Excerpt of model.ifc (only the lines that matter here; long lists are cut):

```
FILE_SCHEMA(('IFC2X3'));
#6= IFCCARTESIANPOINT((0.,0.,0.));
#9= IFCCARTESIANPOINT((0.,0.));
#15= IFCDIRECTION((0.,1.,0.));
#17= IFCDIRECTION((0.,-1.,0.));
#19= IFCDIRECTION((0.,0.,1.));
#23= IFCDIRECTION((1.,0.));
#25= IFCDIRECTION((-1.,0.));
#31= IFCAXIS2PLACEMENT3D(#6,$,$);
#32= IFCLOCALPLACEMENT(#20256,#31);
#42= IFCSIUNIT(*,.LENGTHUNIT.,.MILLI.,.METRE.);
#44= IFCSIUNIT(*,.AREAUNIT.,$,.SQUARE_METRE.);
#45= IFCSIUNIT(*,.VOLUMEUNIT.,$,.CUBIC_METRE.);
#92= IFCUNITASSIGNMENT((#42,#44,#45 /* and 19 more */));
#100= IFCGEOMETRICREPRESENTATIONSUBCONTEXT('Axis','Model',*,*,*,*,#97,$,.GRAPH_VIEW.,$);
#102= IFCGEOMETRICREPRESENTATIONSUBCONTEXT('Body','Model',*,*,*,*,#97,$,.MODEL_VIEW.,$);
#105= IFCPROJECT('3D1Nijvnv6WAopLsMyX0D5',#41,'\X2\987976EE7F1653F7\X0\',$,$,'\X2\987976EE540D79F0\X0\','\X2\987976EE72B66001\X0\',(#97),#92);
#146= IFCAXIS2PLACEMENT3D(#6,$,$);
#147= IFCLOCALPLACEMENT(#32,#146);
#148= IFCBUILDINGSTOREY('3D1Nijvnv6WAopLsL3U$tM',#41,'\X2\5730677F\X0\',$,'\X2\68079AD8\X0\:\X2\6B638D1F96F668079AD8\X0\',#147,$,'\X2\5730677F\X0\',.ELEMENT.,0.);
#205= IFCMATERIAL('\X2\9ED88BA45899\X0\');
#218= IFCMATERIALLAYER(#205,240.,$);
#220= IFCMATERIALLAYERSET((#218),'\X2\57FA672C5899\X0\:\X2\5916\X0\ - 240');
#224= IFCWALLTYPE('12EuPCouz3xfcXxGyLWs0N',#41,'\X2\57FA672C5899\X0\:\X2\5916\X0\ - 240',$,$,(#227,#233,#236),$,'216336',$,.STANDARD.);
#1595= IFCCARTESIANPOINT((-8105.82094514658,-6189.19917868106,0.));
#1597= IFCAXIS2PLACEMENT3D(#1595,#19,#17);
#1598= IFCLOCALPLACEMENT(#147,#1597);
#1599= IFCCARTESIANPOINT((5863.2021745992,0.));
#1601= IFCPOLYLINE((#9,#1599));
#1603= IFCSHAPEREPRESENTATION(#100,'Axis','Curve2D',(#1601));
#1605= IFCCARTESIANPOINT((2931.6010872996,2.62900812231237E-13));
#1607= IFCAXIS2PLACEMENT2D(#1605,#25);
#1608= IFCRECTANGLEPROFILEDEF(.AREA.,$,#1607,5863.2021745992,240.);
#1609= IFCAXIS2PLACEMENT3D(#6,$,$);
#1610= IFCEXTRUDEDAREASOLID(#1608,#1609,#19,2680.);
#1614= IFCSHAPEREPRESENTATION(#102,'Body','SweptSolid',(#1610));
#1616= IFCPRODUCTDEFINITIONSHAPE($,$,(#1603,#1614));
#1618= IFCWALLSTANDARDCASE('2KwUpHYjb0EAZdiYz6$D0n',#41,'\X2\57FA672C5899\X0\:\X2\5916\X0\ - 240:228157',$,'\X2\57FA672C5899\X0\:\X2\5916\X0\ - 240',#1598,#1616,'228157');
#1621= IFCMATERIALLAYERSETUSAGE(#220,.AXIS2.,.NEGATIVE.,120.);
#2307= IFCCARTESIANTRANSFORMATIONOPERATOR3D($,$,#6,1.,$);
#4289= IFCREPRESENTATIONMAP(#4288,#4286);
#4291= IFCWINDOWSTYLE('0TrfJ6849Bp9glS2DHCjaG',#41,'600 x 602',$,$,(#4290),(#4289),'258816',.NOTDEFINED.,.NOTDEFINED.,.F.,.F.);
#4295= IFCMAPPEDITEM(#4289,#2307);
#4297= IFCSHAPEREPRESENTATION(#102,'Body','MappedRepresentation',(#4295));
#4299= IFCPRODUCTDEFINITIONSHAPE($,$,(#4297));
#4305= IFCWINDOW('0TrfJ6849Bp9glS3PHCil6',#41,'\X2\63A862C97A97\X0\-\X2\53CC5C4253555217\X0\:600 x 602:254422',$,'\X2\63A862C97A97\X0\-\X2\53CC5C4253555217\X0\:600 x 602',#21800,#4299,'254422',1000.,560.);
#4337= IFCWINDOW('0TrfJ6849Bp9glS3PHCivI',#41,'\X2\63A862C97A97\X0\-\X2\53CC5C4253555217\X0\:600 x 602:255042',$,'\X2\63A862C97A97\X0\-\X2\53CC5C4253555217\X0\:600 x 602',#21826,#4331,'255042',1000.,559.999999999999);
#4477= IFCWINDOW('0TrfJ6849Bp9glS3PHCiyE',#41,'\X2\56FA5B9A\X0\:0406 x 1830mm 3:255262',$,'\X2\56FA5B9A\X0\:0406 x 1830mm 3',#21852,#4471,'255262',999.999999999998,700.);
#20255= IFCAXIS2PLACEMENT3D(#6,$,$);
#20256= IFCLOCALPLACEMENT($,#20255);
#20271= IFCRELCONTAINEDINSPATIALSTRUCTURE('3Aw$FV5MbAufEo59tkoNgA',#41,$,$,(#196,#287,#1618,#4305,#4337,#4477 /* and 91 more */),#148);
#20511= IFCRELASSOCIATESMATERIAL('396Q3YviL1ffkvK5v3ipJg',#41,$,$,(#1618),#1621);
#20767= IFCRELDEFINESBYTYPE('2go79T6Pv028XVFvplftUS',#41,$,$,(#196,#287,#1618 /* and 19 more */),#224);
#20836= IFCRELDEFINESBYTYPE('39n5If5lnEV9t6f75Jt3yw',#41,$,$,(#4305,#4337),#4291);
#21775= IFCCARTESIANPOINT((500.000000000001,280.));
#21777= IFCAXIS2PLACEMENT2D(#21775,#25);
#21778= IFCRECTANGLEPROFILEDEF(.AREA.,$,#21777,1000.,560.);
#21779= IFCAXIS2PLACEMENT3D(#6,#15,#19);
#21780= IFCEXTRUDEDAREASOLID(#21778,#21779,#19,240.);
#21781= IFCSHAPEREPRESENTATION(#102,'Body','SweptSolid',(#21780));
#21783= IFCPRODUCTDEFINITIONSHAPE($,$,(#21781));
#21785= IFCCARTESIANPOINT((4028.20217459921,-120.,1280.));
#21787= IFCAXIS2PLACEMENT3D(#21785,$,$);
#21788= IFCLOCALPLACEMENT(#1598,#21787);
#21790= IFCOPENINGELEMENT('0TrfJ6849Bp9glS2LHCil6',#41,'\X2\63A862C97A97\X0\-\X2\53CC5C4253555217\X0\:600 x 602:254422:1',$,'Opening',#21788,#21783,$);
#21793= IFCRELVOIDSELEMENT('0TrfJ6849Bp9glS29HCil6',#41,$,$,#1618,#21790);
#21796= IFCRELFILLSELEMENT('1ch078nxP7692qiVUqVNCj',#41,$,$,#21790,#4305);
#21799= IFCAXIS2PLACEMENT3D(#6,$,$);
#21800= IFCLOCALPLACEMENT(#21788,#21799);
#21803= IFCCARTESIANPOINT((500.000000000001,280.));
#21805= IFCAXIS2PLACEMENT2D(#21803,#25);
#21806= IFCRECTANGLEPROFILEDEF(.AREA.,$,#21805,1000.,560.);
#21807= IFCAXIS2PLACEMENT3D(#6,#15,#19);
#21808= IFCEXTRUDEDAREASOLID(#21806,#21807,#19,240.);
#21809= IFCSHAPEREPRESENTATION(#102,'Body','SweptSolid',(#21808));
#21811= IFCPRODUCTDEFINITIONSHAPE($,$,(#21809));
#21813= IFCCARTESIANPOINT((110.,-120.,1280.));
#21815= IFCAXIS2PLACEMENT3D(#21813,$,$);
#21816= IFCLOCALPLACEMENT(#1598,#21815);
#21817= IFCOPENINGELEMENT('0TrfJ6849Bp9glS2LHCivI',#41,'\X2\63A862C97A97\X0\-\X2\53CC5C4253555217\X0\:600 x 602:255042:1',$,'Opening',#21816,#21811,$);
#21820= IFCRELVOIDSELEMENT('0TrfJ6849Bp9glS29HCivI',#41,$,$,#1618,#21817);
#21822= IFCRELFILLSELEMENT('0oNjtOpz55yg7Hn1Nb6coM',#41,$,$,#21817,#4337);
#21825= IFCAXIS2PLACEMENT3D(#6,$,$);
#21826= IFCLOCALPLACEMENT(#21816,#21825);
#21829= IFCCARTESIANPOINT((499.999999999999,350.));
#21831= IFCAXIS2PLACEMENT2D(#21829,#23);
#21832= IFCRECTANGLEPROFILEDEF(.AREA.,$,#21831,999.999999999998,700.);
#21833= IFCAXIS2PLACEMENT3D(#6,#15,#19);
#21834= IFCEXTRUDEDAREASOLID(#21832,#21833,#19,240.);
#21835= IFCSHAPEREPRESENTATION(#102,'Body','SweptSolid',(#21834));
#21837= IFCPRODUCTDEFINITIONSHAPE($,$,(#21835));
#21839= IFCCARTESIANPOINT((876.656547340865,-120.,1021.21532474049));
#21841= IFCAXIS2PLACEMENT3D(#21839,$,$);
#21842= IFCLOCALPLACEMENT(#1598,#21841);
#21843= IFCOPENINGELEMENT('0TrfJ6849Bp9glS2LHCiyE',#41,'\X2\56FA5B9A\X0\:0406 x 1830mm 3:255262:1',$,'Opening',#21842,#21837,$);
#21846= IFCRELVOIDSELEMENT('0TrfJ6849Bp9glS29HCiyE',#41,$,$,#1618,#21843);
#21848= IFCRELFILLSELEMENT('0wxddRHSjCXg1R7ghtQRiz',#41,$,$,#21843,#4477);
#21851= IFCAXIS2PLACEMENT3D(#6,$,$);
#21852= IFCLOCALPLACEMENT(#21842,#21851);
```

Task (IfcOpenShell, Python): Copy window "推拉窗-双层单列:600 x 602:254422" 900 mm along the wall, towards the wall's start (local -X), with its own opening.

```python
import ifcopenshell
import ifcopenshell.api.feature
import ifcopenshell.api.geometry
import ifcopenshell.api.root
import ifcopenshell.geom
import ifcopenshell.util.element
import ifcopenshell.util.placement
import ifcopenshell.util.shape
import ifcopenshell.util.unit

model = ifcopenshell.open("model.ifc")
unit_scale = ifcopenshell.util.unit.calculate_unit_scale(model)
settings = ifcopenshell.geom.settings()


def volume(element):
    """Net volume in cubic metres, openings subtracted."""
    shape = ifcopenshell.geom.create_shape(settings, element)
    return ifcopenshell.util.shape.get_volume(shape.geometry)


def reuse_history(source, copy):
    """copy_class also copies each property set's owner history, people and application; keep the originals."""
    for rel in copy.IsDefinedBy:
        if rel.is_a("IfcRelDefinesByProperties") and (history := rel.RelatingPropertyDefinition.OwnerHistory):
            rel.RelatingPropertyDefinition.OwnerHistory = source.OwnerHistory
            ifcopenshell.util.element.remove_deep2(model, history)


window = model.by_guid("0TrfJ6849Bp9glS3PHCil6")
opening = window.FillsVoids[0].RelatingOpeningElement
wall = opening.VoidsElements[0].RelatingBuildingElement
before = volume(wall)
shift = ifcopenshell.util.placement.get_local_placement(wall.ObjectPlacement)[:3, 0] * -0.9 / unit_scale

# copy_class copies the void relationship, type, container and properties, but no geometry.
new_opening = ifcopenshell.api.root.copy_class(model, product=opening)
new_opening.Representation = ifcopenshell.util.element.copy_deep(
    model, opening.Representation, exclude=["IfcGeometricRepresentationContext", "IfcRepresentationMap"]
)
new_opening.Name = "推拉窗-双层单列:600 x 602"
new_window = ifcopenshell.api.root.copy_class(model, product=window)
new_window.Representation = ifcopenshell.util.element.copy_deep(
    model, window.Representation, exclude=["IfcGeometricRepresentationContext", "IfcRepresentationMap"]
)
new_window.Name = "推拉窗-双层单列:600 x 602"
new_window.Tag = None
reuse_history(window, new_window)
fills = ifcopenshell.api.feature.add_filling(model, opening=new_opening, element=new_window)
fills.OwnerHistory = new_window.OwnerHistory  # required in IFC2X3

for old, new in ((opening, new_opening), (window, new_window)):
    matrix = ifcopenshell.util.placement.get_local_placement(old.ObjectPlacement)
    matrix[:3, 3] += shift
    ifcopenshell.api.geometry.edit_object_placement(model, product=new, matrix=matrix, is_si=False)

after = volume(wall)

print(f"wall volume {before:.3f} -> {after:.3f} m3")

model.write("model_edited.ifc")
```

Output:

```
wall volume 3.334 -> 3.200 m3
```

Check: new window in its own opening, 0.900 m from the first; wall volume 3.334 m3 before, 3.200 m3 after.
